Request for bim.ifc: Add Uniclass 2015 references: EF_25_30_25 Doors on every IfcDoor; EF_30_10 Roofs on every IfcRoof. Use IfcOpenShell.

First a look at what the model holds.

```python
import ifcopenshell

model = ifcopenshell.open("bim.ifc")
print(model.schema)
print("classifications:", [c.Name for c in model.by_type("IfcClassification")])
for ifc_class in ("IfcDoor", "IfcRoof", "IfcStair", "IfcWall", "IfcWindow"):
    print(ifc_class, len(model.by_type(ifc_class)))
```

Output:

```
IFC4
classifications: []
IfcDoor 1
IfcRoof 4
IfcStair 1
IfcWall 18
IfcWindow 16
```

```python
import ifcopenshell
import ifcopenshell.api.classification

model = ifcopenshell.open("bim.ifc")

system = ifcopenshell.api.classification.add_classification(model, classification="Uniclass 2015")

codes = {
    "IfcDoor": ("EF_25_30_25", "Doors"),
    "IfcRoof": ("EF_30_10", "Roofs"),
}
for ifc_class, (code, name) in codes.items():
    products = model.by_type(ifc_class)
    ifcopenshell.api.classification.add_reference(
        model, products=products, classification=system, identification=code, name=name
    )
    print(code, len(products))

model.write("bim_rev.ifc")
```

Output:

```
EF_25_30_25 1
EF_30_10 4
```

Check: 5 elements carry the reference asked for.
